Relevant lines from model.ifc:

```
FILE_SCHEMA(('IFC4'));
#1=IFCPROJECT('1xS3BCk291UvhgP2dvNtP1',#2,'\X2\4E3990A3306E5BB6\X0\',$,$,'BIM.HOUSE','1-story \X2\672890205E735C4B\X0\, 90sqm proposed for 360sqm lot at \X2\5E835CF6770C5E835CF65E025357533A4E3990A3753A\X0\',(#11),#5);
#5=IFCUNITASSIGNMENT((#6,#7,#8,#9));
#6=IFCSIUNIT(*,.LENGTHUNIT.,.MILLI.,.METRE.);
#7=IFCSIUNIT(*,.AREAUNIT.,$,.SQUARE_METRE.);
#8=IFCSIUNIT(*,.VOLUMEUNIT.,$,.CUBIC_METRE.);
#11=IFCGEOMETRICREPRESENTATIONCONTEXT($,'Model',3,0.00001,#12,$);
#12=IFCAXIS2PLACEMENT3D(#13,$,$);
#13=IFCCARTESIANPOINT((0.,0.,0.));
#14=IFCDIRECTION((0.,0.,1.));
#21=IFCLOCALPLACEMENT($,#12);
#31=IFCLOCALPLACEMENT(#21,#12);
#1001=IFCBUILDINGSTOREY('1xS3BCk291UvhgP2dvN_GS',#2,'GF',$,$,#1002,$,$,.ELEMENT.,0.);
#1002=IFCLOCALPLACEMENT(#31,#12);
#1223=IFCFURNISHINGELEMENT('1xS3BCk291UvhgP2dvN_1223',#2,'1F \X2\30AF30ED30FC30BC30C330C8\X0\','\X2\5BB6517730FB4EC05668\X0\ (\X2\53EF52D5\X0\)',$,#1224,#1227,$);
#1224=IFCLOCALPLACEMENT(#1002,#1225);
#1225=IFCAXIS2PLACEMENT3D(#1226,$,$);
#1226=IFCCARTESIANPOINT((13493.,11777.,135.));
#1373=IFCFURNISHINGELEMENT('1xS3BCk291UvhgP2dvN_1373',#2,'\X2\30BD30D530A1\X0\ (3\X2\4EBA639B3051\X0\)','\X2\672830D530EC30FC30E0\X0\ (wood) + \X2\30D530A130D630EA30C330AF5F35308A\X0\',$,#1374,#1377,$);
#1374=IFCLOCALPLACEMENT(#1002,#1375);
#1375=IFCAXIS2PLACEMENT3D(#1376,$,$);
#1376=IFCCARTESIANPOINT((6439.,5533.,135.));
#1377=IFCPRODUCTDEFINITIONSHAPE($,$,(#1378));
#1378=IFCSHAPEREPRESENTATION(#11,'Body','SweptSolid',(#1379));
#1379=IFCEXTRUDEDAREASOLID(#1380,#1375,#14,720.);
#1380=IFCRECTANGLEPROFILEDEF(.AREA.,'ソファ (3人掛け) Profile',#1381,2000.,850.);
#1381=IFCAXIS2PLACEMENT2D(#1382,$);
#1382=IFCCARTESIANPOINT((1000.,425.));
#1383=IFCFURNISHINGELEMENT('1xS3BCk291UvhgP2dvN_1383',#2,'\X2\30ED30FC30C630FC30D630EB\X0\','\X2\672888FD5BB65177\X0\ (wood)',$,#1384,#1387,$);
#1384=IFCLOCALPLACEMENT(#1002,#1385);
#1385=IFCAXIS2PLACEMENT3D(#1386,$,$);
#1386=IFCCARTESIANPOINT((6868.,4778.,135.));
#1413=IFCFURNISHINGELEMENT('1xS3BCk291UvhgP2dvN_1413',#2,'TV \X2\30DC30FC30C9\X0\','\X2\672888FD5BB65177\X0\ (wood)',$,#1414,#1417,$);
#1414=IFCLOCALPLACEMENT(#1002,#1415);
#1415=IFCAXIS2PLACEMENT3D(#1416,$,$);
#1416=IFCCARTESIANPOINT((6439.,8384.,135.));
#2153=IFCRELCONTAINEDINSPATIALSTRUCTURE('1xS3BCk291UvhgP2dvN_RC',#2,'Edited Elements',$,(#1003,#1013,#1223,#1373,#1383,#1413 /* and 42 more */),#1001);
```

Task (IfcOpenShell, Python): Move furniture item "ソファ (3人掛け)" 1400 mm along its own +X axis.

```python
import ifcopenshell
import ifcopenshell.api.geometry
import ifcopenshell.util.placement
import ifcopenshell.util.unit

model = ifcopenshell.open("model.ifc")
unit_scale = ifcopenshell.util.unit.calculate_unit_scale(model)

item = model.by_guid("1xS3BCk291UvhgP2dvN_1373")
matrix = ifcopenshell.util.placement.get_local_placement(item.ObjectPlacement)
matrix[:3, 3] += matrix[:3, 0] * 1.4 / unit_scale
ifcopenshell.api.geometry.edit_object_placement(model, product=item, matrix=matrix, is_si=False)

print(ifcopenshell.util.placement.get_local_placement(item.ObjectPlacement).round(3) + 0.0)

model.write("model_rev.ifc")
```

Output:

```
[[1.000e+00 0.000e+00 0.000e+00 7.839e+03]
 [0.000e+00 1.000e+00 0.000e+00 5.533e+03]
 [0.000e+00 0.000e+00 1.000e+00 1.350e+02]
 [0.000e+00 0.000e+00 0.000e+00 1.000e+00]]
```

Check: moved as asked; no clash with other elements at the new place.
